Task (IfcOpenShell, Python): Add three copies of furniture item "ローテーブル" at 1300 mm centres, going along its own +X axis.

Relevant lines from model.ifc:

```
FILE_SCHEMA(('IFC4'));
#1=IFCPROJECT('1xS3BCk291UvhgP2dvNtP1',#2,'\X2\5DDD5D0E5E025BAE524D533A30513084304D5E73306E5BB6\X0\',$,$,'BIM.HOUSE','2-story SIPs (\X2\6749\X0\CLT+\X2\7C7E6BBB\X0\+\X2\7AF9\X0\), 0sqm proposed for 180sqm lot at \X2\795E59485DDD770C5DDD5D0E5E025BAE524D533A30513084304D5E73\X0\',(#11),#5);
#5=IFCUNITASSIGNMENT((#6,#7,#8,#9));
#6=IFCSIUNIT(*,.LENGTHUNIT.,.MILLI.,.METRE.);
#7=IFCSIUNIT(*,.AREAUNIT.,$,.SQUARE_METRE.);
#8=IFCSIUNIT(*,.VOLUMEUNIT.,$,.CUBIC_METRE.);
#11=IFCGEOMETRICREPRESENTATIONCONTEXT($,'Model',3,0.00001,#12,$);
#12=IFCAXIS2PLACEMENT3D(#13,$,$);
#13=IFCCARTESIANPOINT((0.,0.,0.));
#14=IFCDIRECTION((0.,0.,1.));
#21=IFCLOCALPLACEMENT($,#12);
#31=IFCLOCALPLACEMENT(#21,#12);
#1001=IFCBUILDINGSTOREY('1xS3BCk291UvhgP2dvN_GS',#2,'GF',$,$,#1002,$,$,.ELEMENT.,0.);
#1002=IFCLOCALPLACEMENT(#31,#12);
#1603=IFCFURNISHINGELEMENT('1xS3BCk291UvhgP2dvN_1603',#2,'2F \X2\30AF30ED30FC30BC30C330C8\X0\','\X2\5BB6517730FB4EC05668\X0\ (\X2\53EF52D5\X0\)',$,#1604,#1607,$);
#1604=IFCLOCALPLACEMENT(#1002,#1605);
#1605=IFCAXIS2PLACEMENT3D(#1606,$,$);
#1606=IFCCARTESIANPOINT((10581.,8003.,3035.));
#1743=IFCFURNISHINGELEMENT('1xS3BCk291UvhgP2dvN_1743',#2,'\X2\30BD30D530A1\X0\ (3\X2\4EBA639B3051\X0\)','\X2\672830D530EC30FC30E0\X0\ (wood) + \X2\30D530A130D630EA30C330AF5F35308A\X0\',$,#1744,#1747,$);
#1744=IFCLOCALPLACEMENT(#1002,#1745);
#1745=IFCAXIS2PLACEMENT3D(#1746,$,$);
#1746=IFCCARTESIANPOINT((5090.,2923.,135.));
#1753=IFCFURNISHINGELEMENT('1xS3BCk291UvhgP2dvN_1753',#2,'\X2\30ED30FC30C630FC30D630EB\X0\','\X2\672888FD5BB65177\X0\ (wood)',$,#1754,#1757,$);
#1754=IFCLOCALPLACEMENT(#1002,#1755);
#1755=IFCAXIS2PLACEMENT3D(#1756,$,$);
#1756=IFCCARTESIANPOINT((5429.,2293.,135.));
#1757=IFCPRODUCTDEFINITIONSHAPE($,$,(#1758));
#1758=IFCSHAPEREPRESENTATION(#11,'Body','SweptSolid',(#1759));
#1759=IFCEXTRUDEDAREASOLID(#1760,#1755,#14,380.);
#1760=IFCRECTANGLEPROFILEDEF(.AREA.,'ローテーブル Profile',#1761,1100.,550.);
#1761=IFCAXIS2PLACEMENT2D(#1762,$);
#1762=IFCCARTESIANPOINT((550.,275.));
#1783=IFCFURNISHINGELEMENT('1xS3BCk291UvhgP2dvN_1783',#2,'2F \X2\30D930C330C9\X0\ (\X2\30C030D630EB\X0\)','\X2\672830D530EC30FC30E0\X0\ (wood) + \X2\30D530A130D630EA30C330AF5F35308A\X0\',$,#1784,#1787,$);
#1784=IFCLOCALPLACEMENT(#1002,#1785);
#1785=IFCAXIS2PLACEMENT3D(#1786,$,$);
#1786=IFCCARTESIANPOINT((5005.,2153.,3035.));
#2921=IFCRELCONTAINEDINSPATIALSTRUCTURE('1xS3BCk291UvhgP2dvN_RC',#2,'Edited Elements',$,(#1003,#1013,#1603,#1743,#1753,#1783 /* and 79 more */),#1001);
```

```python
import ifcopenshell
import ifcopenshell.api.geometry
import ifcopenshell.api.root
import ifcopenshell.util.element
import ifcopenshell.util.placement

model = ifcopenshell.open("model.ifc")


def reuse_history(source, copy):
    """copy_class also copies each property set's owner history, people and application; keep the originals."""
    for rel in copy.IsDefinedBy:
        if rel.is_a("IfcRelDefinesByProperties") and (history := rel.RelatingPropertyDefinition.OwnerHistory):
            rel.RelatingPropertyDefinition.OwnerHistory = source.OwnerHistory
            ifcopenshell.util.element.remove_deep2(model, history)


source = model.by_guid("1xS3BCk291UvhgP2dvN_1753")
base = ifcopenshell.util.placement.get_local_placement(source.ObjectPlacement)
step = base[:3, 0] * 1300.0

for i in range(1, 4):
    copy = ifcopenshell.api.root.copy_class(model, product=source)
    copy.Representation = ifcopenshell.util.element.copy_deep(
        model, source.Representation, exclude=["IfcGeometricRepresentationContext", "IfcRepresentationMap"]
    )
    reuse_history(source, copy)
    matrix = base.copy()
    matrix[:3, 3] += i * step
    print("added at", matrix[:3, 3].round(3) + 0.0)
    ifcopenshell.api.geometry.edit_object_placement(model, product=copy, matrix=matrix, is_si=False)

model.write("model_edited.ifc")
```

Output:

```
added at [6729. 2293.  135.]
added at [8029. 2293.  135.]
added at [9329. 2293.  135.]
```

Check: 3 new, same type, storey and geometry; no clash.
